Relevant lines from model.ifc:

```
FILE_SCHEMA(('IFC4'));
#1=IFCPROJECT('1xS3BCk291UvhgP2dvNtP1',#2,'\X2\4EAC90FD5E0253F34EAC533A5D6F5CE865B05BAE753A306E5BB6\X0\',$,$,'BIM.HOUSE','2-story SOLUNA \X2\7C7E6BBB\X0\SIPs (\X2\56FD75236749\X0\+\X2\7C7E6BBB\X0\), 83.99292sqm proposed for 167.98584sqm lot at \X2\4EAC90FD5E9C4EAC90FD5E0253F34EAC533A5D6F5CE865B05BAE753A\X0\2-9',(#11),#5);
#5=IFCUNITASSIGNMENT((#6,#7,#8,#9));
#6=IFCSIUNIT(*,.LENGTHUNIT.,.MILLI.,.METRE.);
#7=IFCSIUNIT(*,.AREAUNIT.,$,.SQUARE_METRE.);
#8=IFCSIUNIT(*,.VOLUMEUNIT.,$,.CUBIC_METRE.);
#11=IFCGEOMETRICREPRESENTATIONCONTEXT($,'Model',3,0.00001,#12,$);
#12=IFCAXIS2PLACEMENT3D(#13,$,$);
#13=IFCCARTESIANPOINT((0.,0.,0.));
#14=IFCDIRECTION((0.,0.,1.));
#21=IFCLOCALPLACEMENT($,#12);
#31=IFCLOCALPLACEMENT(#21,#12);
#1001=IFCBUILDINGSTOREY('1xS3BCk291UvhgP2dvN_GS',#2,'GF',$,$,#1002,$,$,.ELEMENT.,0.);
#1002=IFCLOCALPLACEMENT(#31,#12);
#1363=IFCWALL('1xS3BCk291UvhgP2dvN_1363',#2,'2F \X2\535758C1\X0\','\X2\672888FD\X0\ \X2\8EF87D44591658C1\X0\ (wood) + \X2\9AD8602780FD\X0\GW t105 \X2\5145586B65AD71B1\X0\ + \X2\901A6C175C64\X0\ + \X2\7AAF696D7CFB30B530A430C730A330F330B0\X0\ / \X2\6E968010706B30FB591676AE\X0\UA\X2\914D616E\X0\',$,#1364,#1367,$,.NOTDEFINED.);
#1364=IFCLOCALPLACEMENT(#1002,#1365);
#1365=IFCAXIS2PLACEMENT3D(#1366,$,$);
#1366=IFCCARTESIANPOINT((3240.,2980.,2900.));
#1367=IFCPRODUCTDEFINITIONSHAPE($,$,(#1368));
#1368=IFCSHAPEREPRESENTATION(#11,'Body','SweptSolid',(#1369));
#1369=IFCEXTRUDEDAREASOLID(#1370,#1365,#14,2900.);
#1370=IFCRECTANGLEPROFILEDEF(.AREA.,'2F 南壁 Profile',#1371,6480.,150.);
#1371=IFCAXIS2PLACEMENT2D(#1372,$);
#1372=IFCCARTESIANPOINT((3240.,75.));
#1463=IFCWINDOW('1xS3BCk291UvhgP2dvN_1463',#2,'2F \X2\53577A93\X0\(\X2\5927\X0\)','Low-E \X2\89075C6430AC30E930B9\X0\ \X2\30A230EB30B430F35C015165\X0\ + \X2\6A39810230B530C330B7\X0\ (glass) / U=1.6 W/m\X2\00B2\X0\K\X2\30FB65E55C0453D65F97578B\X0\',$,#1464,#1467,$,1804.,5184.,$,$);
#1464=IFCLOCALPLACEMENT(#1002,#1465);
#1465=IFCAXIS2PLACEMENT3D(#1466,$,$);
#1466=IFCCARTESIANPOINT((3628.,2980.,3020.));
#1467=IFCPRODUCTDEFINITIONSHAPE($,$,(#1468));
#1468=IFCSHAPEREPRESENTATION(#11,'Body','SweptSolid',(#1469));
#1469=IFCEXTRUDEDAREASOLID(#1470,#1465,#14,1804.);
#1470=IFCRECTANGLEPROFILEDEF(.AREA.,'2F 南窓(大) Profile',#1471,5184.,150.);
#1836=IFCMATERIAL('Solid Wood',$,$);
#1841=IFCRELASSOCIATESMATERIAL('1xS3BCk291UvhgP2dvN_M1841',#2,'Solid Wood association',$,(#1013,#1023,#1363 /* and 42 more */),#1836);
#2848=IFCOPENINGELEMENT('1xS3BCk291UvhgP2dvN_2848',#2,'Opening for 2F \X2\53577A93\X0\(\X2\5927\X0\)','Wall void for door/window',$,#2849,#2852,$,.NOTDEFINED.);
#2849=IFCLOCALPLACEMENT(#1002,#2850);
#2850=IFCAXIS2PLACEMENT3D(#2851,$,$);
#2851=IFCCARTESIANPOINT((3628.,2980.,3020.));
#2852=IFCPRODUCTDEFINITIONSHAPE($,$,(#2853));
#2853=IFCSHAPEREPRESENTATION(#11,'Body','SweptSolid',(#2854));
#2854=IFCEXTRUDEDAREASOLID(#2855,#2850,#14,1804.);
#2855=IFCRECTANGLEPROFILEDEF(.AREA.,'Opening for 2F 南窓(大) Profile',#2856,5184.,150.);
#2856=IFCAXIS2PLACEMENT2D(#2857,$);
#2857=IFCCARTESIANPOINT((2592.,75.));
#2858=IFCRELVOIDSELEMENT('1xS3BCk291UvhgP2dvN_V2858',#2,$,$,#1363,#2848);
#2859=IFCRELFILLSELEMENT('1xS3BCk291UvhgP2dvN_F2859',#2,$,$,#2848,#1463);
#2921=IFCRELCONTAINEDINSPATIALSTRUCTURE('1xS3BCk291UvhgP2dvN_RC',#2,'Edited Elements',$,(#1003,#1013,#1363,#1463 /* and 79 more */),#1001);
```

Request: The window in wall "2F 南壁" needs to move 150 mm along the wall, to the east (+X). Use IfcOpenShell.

```python
import ifcopenshell
import ifcopenshell.api.geometry
import ifcopenshell.util.placement
import ifcopenshell.util.unit

model = ifcopenshell.open("model.ifc")
unit_scale = ifcopenshell.util.unit.calculate_unit_scale(model)

window = model.by_id(1463)
opening = window.FillsVoids[0].RelatingOpeningElement
wall = opening.VoidsElements[0].RelatingBuildingElement

wall_matrix = ifcopenshell.util.placement.get_local_placement(wall.ObjectPlacement)
shift = wall_matrix[:3, 0] * 0.15 / unit_scale
before = ifcopenshell.util.placement.get_local_placement(window.ObjectPlacement)[:3, 3].copy()

# The window is not placed relative to its opening, so move both.
for product in (opening, window):
    matrix = ifcopenshell.util.placement.get_local_placement(product.ObjectPlacement)
    matrix[:3, 3] += shift
    ifcopenshell.api.geometry.edit_object_placement(model, product=product, matrix=matrix, is_si=False)

after = ifcopenshell.util.placement.get_local_placement(window.ObjectPlacement)[:3, 3]
print("window moved by", (after - before).round(3) + 0.0)

model.write("model_updated.ifc")
```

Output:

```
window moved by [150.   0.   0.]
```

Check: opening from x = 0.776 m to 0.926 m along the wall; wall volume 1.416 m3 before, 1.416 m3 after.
